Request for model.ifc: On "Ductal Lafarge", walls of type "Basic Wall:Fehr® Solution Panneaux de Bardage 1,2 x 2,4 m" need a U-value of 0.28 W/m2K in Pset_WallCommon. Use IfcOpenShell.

First a look at what the model holds.

```python
import ifcopenshell
import ifcopenshell.util.element

model = ifcopenshell.open("model.ifc")
print(model.schema)
storey = next(s for s in model.by_type("IfcBuildingStorey") if s.Name == "Ductal Lafarge")
walls = [e for e in ifcopenshell.util.element.get_decomposition(storey) if e.is_a("IfcWall")]
seen = {}
for e in walls:
    element_type = ifcopenshell.util.element.get_type(e)
    key = (element_type.Name if element_type != e and element_type else None, ifcopenshell.util.element.get_pset(e, "Pset_WallCommon", "ThermalTransmittance"))
    seen[key] = seen.get(key, 0) + 1
for (name, value), count in sorted(seen.items(), key=str):
    print(count, "x", name, "|", value)
```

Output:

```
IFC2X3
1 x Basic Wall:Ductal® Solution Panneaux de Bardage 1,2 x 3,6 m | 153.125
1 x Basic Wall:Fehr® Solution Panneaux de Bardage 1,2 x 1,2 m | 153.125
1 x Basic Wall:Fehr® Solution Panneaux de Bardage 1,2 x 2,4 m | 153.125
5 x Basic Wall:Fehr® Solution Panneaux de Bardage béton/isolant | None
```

```python
import ifcopenshell
import ifcopenshell.api.pset
import ifcopenshell.util.element

model = ifcopenshell.open("model.ifc")

storey = next(s for s in model.by_type("IfcBuildingStorey") if s.Name == "Ductal Lafarge")
walls = [e for e in ifcopenshell.util.element.get_decomposition(storey) if e.is_a("IfcWall")]

count = 0
for e in walls:
    element_type = ifcopenshell.util.element.get_type(e)
    if element_type in (None, e) or element_type.Name != "Basic Wall:Fehr® Solution Panneaux de Bardage 1,2 x 2,4 m":
        continue
    # add_pset returns the element's existing set when there is one.
    pset = ifcopenshell.api.pset.add_pset(model, product=e, name="Pset_WallCommon")
    ifcopenshell.api.pset.edit_pset(model, pset=pset, properties={"ThermalTransmittance": 0.28})
    count += 1

print(count, "walls updated")

model.write("model_v2.ifc")
```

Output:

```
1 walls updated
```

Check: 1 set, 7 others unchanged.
